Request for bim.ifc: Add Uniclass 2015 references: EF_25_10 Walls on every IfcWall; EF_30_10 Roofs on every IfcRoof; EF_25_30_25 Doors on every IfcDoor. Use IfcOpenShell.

First a look at what the model holds.

```python
import ifcopenshell

model = ifcopenshell.open("bim.ifc")
print(model.schema)
print("classifications:", [c.Name for c in model.by_type("IfcClassification")])
for ifc_class in ("IfcDoor", "IfcRoof", "IfcStair", "IfcWall", "IfcWindow"):
    print(ifc_class, len(model.by_type(ifc_class)))
```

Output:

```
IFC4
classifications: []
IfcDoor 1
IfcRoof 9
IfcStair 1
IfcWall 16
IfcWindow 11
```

```python
import ifcopenshell
import ifcopenshell.api.classification

model = ifcopenshell.open("bim.ifc")

system = ifcopenshell.api.classification.add_classification(model, classification="Uniclass 2015")

codes = {
    "IfcWall": ("EF_25_10", "Walls"),
    "IfcRoof": ("EF_30_10", "Roofs"),
    "IfcDoor": ("EF_25_30_25", "Doors"),
}
for ifc_class, (code, name) in codes.items():
    products = model.by_type(ifc_class)
    ifcopenshell.api.classification.add_reference(
        model, products=products, classification=system, identification=code, name=name
    )
    print(code, len(products))

model.write("bim_v2.ifc")
```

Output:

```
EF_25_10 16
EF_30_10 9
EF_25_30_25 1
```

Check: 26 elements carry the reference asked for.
